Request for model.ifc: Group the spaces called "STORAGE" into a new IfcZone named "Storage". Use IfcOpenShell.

First a look at what the model holds.

```python
import ifcopenshell

model = ifcopenshell.open("model.ifc")
print(model.schema)
seen = {}
for space in model.by_type("IfcSpace"):
    seen[space.LongName] = seen.get(space.LongName, 0) + 1
for name, count in sorted(seen.items(), key=str):
    print(count, "x", name)
print("zones:", [z.Name for z in model.by_type("IfcZone")][:20])
```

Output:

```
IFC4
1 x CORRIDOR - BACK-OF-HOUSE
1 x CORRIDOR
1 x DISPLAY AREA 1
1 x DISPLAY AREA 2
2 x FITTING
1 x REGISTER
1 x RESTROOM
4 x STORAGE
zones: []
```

```python
import ifcopenshell
import ifcopenshell.api.group
import ifcopenshell.api.root

model = ifcopenshell.open("model.ifc")

names = {"STORAGE"}
spaces = [s for s in model.by_type("IfcSpace") if s.LongName in names]

zone = ifcopenshell.api.root.create_entity(model, ifc_class="IfcZone", name="Storage")
ifcopenshell.api.group.assign_group(model, products=spaces, group=zone)
print(len(spaces), "spaces in", zone.Name)

model.write("model_v2.ifc")
```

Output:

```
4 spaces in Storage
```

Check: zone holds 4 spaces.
